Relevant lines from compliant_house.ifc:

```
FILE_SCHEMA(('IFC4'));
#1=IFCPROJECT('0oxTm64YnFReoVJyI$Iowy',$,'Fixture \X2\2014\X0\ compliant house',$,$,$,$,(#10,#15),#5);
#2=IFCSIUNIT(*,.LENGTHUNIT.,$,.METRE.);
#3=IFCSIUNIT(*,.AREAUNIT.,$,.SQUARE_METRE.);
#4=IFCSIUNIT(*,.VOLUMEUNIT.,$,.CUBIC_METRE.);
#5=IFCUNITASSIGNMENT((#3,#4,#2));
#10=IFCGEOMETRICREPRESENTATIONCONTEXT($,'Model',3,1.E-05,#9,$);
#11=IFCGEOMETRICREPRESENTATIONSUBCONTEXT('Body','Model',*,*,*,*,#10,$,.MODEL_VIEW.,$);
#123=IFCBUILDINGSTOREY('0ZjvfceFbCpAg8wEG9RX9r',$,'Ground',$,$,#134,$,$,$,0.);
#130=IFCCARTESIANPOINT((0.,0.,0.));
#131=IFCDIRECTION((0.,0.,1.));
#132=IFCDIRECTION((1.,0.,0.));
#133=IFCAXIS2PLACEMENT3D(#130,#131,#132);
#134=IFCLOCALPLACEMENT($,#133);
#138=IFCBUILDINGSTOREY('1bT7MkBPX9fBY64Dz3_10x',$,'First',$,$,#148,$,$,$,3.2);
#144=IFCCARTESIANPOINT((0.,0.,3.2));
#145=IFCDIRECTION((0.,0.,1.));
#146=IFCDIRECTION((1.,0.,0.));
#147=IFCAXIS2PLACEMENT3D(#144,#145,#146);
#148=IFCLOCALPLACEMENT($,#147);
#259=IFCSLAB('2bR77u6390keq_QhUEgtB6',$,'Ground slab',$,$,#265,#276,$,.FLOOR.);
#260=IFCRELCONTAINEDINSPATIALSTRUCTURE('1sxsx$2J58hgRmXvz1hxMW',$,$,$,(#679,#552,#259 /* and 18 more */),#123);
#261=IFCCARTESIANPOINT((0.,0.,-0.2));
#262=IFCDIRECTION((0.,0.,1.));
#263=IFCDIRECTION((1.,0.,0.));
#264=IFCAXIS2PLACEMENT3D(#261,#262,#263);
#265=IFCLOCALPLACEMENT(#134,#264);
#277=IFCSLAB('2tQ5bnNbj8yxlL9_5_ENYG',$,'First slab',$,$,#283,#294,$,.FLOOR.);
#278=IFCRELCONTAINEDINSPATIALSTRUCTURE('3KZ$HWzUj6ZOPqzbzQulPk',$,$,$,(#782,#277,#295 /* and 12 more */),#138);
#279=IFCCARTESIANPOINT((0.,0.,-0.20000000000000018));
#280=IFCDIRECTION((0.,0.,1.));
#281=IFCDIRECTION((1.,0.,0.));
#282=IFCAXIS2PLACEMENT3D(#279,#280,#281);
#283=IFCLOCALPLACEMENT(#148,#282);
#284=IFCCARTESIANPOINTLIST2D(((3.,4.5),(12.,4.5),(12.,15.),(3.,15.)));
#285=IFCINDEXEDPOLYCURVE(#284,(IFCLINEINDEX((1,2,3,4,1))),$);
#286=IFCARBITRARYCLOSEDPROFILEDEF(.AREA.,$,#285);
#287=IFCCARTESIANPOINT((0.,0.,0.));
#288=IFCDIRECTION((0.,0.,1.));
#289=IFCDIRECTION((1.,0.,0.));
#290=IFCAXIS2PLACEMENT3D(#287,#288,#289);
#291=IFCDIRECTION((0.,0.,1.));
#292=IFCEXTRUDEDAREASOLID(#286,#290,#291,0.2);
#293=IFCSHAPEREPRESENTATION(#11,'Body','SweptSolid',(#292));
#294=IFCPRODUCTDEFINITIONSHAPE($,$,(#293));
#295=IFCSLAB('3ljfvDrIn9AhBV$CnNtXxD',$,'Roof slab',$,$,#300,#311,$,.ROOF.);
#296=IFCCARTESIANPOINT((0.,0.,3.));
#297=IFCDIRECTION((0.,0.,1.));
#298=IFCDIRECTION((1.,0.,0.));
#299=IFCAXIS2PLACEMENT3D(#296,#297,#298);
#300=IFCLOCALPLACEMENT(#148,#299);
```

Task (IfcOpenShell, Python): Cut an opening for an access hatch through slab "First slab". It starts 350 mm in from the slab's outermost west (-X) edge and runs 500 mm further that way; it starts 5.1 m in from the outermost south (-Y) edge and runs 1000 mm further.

```python
import numpy as np
import ifcopenshell
import ifcopenshell.api.feature
import ifcopenshell.api.geometry
import ifcopenshell.api.root
import ifcopenshell.geom
import ifcopenshell.util.placement
import ifcopenshell.util.representation
import ifcopenshell.util.shape
import ifcopenshell.util.unit

model = ifcopenshell.open("compliant_house.ifc")
unit_scale = ifcopenshell.util.unit.calculate_unit_scale(model)
settings = ifcopenshell.geom.settings()


def volume(element):
    """Net volume in cubic metres, openings subtracted."""
    shape = ifcopenshell.geom.create_shape(settings, element)
    return ifcopenshell.util.shape.get_volume(shape.geometry)


slab = model.by_guid("2tQ5bnNbj8yxlL9_5_ENYG")
before = volume(slab)

# Extent in the slab's own axes, in metres. The edges named are its -X and -Y sides.
slab_shape = ifcopenshell.geom.create_shape(settings, slab)
vertices = ifcopenshell.util.shape.get_vertices(slab_shape.geometry)
x_min, y_min, bottom = vertices.min(axis=0)
top = vertices[:, 2].max()

opening = ifcopenshell.api.root.create_entity(model, ifc_class="IfcOpeningElement", name="Access hatch opening", predefined_type="OPENING")
context = ifcopenshell.util.representation.get_context(model, "Model", "Body", "MODEL_VIEW")
width, depth = 0.5, 1
outline = [(0.0, 0.0), (width, 0.0), (width, depth), (0.0, depth), (0.0, 0.0)]
# Overshoot both faces by 50 mm so the cut is clean.
shape = ifcopenshell.api.geometry.add_slab_representation(
    model, context=context, depth=top - bottom + 0.1, polyline=outline
)
ifcopenshell.api.geometry.assign_representation(model, product=opening, representation=shape)

matrix = ifcopenshell.util.placement.get_local_placement(slab.ObjectPlacement)
matrix[:, 3] = matrix @ np.append(np.array([x_min + 0.35, y_min + 5.1, bottom - 0.05]) / unit_scale, 1.0)
ifcopenshell.api.geometry.edit_object_placement(model, product=opening, matrix=matrix, is_si=False)
ifcopenshell.api.feature.add_feature(model, feature=opening, element=slab)

after = volume(slab)

print(f"slab volume {before:.3f} -> {after:.3f} m3")

model.write("compliant_house_edited.ifc")
```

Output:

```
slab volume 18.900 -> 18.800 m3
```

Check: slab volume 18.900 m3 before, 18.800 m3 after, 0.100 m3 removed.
